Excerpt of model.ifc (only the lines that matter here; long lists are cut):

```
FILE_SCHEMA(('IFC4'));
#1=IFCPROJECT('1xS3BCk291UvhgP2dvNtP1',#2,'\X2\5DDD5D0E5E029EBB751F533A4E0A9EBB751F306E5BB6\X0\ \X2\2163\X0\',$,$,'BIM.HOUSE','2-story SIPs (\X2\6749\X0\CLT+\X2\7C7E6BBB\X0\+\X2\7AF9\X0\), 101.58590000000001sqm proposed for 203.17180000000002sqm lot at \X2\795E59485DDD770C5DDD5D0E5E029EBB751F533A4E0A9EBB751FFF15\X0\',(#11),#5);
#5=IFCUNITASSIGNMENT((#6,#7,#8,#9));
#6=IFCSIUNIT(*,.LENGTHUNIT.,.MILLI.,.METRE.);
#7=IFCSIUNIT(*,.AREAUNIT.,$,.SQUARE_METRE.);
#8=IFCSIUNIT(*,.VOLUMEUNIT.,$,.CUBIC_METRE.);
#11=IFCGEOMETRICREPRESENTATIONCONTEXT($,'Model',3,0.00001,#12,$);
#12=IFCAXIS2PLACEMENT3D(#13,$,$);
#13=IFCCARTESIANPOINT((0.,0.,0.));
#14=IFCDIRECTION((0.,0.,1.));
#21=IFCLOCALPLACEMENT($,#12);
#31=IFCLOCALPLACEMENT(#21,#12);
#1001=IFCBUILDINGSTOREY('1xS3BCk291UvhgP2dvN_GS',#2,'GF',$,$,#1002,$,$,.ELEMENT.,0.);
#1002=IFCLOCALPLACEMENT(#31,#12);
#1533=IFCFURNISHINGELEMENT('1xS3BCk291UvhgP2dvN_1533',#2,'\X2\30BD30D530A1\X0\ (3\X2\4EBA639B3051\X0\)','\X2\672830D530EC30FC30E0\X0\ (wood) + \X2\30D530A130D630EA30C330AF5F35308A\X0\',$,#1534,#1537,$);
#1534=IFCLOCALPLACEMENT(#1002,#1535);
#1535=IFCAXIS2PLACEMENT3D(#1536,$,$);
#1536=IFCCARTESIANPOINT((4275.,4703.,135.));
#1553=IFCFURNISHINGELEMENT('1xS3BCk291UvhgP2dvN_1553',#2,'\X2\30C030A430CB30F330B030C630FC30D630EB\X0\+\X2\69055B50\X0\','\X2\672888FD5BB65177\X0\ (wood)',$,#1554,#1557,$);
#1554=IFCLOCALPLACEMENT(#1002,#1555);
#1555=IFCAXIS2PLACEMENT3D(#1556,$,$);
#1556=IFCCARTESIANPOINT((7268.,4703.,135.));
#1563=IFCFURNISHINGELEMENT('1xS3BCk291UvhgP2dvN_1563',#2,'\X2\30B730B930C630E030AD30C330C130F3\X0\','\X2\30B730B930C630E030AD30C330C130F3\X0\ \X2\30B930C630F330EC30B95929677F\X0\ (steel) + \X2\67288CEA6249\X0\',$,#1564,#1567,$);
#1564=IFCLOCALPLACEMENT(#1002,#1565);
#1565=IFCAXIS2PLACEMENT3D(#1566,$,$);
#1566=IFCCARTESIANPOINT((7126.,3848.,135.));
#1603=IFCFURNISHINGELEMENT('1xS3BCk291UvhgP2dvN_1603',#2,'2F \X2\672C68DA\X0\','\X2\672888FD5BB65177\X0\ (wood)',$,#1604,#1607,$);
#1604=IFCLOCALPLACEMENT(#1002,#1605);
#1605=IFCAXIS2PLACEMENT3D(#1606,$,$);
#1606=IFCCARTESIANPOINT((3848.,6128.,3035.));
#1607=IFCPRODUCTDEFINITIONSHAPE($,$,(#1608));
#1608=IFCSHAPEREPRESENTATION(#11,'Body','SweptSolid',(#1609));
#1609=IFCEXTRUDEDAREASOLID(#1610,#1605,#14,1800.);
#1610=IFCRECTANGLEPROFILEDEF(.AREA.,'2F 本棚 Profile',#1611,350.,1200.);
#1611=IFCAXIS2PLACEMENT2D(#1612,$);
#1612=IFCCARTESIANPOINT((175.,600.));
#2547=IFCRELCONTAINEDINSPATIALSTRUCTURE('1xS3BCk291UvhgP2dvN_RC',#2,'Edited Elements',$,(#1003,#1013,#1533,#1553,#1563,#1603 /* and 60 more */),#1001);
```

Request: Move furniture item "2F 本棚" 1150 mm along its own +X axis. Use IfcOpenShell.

```python
import ifcopenshell
import ifcopenshell.api.geometry
import ifcopenshell.util.placement
import ifcopenshell.util.unit

model = ifcopenshell.open("model.ifc")
unit_scale = ifcopenshell.util.unit.calculate_unit_scale(model)

item = model.by_id(1603)
matrix = ifcopenshell.util.placement.get_local_placement(item.ObjectPlacement)
matrix[:3, 3] += matrix[:3, 0] * 1.15 / unit_scale
ifcopenshell.api.geometry.edit_object_placement(model, product=item, matrix=matrix, is_si=False)

print(ifcopenshell.util.placement.get_local_placement(item.ObjectPlacement).round(3) + 0.0)

model.write("model_edited.ifc")
```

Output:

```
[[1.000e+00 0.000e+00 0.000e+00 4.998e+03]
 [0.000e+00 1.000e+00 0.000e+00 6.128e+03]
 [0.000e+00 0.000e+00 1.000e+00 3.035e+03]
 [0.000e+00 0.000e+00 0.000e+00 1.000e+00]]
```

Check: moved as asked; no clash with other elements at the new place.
